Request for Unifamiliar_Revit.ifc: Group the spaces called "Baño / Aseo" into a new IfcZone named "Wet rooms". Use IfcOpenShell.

First a look at what the model holds.

```python
import ifcopenshell

model = ifcopenshell.open("Unifamiliar_Revit.ifc")
print(model.schema)
seen = {}
for space in model.by_type("IfcSpace"):
    seen[space.LongName] = seen.get(space.LongName, 0) + 1
for name, count in sorted(seen.items(), key=str):
    print(count, "x", name)
print("zones:", [z.Name for z in model.by_type("IfcZone")][:20])
```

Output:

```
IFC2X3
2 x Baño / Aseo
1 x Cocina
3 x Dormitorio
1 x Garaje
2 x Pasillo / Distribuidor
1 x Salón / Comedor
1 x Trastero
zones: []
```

```python
import ifcopenshell
import ifcopenshell.api.group
import ifcopenshell.api.root

model = ifcopenshell.open("Unifamiliar_Revit.ifc")

names = {"Baño / Aseo"}
spaces = [s for s in model.by_type("IfcSpace") if s.LongName in names]

zone = ifcopenshell.api.root.create_entity(model, ifc_class="IfcZone", name="Wet rooms")
ifcopenshell.api.group.assign_group(model, products=spaces, group=zone)
print(len(spaces), "spaces in", zone.Name)

model.write("Unifamiliar_Revit_rev.ifc")
```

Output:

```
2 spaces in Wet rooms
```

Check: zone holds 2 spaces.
